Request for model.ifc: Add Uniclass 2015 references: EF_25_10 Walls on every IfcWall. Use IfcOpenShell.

First a look at what the model holds.

```python
import ifcopenshell

model = ifcopenshell.open("model.ifc")
print(model.schema)
print("classifications:", [c.Name for c in model.by_type("IfcClassification")])
for ifc_class in ("IfcDoor", "IfcRoof", "IfcStair", "IfcWall", "IfcWindow"):
    print(ifc_class, len(model.by_type(ifc_class)))
```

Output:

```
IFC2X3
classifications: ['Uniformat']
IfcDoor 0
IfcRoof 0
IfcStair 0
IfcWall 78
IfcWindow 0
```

```python
import ifcopenshell
import ifcopenshell.api.classification

model = ifcopenshell.open("model.ifc")

# IFC2X3 requires Source and Edition and has no link from the project to the system.
system = model.create_entity("IfcClassification", Source="NBS", Edition="2015", Name="Uniclass 2015")

codes = {
    "IfcWall": ("EF_25_10", "Walls"),
}
for ifc_class, (code, name) in codes.items():
    products = model.by_type(ifc_class)
    ifcopenshell.api.classification.add_reference(
        model, products=products, classification=system, identification=code, name=name
    )
    print(code, len(products))

model.write("model_updated.ifc")
```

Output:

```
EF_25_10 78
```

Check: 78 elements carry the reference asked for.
